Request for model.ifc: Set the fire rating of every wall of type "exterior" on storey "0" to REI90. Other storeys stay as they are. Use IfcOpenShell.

First a look at what the model holds.

```python
import ifcopenshell
import ifcopenshell.util.element

model = ifcopenshell.open("model.ifc")
print(model.schema)
storey = next(s for s in model.by_type("IfcBuildingStorey") if s.Name == "0")
walls = [e for e in ifcopenshell.util.element.get_decomposition(storey) if e.is_a("IfcWall")]
seen = {}
for e in walls:
    element_type = ifcopenshell.util.element.get_type(e)
    key = (element_type.Name if element_type != e and element_type else None, ifcopenshell.util.element.get_pset(e, "Pset_WallCommon", "FireRating"))
    seen[key] = seen.get(key, 0) + 1
for (name, value), count in sorted(seen.items(), key=str):
    print(count, "x", name, "|", value)
```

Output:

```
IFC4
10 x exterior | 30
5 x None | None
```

```python
import ifcopenshell
import ifcopenshell.api.pset
import ifcopenshell.util.element

model = ifcopenshell.open("model.ifc")

storey = next(s for s in model.by_type("IfcBuildingStorey") if s.Name == "0")
walls = [e for e in ifcopenshell.util.element.get_decomposition(storey) if e.is_a("IfcWall")]

count = 0
for e in walls:
    element_type = ifcopenshell.util.element.get_type(e)
    if element_type in (None, e) or element_type.Name != "exterior":
        continue
    # add_pset returns the element's existing set when there is one.
    pset = ifcopenshell.api.pset.add_pset(model, product=e, name="Pset_WallCommon")
    ifcopenshell.api.pset.edit_pset(model, pset=pset, properties={"FireRating": "REI90"})
    count += 1

print(count, "walls updated")

model.write("model_v2.ifc")
```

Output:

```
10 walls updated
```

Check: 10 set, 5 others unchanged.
